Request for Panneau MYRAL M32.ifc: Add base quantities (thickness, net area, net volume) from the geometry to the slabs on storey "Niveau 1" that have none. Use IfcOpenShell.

First a look at what the model holds.

```python
import ifcopenshell
import ifcopenshell.util.element
import ifcopenshell.util.unit

model = ifcopenshell.open("Panneau MYRAL M32.ifc")
print(model.schema)
for unit_type in ("LENGTHUNIT", "AREAUNIT", "VOLUMEUNIT"):
    print(unit_type, ifcopenshell.util.unit.calculate_unit_scale(model, unit_type))
storey = next(s for s in model.by_type("IfcBuildingStorey") if s.Name == "Niveau 1")
slabs = [e for e in ifcopenshell.util.element.get_decomposition(storey) if e.is_a("IfcSlab")]
for e in sorted(slabs, key=lambda e: e.id()):
    print(e.id(), e.is_a(), e.Name, list(ifcopenshell.util.element.get_psets(e, qtos_only=True)), sep=" | ")
```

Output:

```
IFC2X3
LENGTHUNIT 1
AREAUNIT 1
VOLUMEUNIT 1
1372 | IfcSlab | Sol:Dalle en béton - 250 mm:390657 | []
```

```python
import ifcopenshell
import ifcopenshell.api.pset
import ifcopenshell.geom
import ifcopenshell.util.element
import ifcopenshell.util.shape
import ifcopenshell.util.unit

model = ifcopenshell.open("Panneau MYRAL M32.ifc")
unit_scale = ifcopenshell.util.unit.calculate_unit_scale(model)
area_scale = ifcopenshell.util.unit.calculate_unit_scale(model, "AREAUNIT")
volume_scale = ifcopenshell.util.unit.calculate_unit_scale(model, "VOLUMEUNIT")
settings = ifcopenshell.geom.settings()

storey = next(s for s in model.by_type("IfcBuildingStorey") if s.Name == "Niveau 1")
slabs = [e for e in ifcopenshell.util.element.get_decomposition(storey) if e.is_a("IfcSlab")]

for e in sorted(slabs, key=lambda e: e.id()):
    if ifcopenshell.util.element.get_psets(e, qtos_only=True, should_inherit=False):
        continue
    # Geometry comes back in metres, in the element's own axes.
    shape = ifcopenshell.geom.create_shape(settings, e)
    values = {
        "Width": ifcopenshell.util.shape.get_z(shape.geometry) / unit_scale,
        "NetArea": ifcopenshell.util.shape.get_footprint_area(shape.geometry) / area_scale,
        "NetVolume": ifcopenshell.util.shape.get_volume(shape.geometry) / volume_scale,
    }
    qto = ifcopenshell.api.pset.add_qto(model, product=e, name="BaseQuantities")
    ifcopenshell.api.pset.edit_qto(model, qto=qto, properties=values)
    print(e.id(), {k: round(v, 3) for k, v in values.items()})

model.write("Panneau MYRAL M32_v2.ifc")
```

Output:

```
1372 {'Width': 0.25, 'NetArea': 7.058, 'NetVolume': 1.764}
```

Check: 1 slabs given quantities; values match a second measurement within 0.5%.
